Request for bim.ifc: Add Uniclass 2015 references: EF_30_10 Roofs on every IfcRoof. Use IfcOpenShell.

First a look at what the model holds.

```python
import ifcopenshell

model = ifcopenshell.open("bim.ifc")
print(model.schema)
print("classifications:", [c.Name for c in model.by_type("IfcClassification")])
for ifc_class in ("IfcDoor", "IfcRoof", "IfcStair", "IfcWall", "IfcWindow"):
    print(ifc_class, len(model.by_type(ifc_class)))
```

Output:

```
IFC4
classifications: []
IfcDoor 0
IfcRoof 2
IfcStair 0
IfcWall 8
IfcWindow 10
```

```python
import ifcopenshell
import ifcopenshell.api.classification

model = ifcopenshell.open("bim.ifc")

system = ifcopenshell.api.classification.add_classification(model, classification="Uniclass 2015")

codes = {
    "IfcRoof": ("EF_30_10", "Roofs"),
}
for ifc_class, (code, name) in codes.items():
    products = model.by_type(ifc_class)
    ifcopenshell.api.classification.add_reference(
        model, products=products, classification=system, identification=code, name=name
    )
    print(code, len(products))

model.write("bim_updated.ifc")
```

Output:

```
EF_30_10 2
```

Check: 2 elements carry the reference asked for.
